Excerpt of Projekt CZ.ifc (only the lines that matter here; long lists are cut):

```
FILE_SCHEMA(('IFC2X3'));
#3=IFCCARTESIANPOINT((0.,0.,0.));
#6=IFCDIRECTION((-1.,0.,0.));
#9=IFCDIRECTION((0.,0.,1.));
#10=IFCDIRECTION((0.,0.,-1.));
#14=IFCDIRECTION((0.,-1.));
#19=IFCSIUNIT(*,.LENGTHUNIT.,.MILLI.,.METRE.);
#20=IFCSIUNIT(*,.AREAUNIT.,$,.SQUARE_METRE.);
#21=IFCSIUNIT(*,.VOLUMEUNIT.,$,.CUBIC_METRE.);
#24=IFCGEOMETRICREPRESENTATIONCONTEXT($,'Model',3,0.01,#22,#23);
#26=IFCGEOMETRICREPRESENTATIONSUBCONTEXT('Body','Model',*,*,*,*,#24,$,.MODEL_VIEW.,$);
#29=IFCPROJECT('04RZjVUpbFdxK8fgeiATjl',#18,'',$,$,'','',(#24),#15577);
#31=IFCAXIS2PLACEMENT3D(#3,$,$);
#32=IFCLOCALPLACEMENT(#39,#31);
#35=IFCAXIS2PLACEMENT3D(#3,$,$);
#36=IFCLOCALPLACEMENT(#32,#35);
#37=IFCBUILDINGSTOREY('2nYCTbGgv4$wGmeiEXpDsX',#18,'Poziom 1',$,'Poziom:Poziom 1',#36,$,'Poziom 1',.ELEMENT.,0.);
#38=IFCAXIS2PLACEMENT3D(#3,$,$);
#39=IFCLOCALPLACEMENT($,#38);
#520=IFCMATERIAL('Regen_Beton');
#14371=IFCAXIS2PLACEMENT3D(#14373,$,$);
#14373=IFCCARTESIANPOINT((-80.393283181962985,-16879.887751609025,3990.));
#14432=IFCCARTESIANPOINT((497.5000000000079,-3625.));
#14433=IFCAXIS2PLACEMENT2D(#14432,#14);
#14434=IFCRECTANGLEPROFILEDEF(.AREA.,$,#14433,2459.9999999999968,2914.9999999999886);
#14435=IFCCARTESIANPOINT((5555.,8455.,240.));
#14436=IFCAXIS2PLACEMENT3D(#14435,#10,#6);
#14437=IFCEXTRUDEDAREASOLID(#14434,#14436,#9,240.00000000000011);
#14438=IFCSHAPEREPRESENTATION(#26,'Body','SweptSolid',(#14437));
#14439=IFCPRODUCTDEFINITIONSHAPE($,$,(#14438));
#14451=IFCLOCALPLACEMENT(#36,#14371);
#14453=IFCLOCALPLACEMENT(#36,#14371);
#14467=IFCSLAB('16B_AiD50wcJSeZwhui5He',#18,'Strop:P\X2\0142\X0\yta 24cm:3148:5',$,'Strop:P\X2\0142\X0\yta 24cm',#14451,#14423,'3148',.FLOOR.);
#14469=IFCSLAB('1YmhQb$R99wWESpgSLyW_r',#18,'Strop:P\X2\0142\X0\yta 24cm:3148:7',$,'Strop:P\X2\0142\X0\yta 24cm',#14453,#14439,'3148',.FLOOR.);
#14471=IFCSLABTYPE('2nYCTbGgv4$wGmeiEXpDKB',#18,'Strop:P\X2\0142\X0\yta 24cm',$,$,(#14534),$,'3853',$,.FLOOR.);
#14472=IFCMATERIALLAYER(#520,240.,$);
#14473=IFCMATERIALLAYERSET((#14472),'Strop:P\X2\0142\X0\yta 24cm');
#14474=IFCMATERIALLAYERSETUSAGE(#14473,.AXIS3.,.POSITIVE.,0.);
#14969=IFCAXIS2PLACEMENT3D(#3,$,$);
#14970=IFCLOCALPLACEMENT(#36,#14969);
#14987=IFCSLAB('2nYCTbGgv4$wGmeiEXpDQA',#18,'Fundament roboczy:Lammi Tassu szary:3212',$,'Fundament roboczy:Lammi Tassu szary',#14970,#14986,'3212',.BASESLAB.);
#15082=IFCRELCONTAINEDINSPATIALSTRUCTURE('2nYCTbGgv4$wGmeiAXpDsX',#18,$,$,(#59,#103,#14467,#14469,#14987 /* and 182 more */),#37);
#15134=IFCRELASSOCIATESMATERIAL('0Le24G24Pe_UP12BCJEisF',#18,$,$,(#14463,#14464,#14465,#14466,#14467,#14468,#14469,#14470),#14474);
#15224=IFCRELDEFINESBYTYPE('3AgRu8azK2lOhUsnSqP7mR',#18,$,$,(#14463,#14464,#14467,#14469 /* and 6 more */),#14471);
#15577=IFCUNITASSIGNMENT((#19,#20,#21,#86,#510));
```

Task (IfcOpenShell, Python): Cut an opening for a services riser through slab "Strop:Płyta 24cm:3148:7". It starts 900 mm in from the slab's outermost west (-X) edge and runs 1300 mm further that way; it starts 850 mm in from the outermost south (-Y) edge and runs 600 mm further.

```python
import numpy as np
import ifcopenshell
import ifcopenshell.api.feature
import ifcopenshell.api.geometry
import ifcopenshell.api.root
import ifcopenshell.geom
import ifcopenshell.util.placement
import ifcopenshell.util.representation
import ifcopenshell.util.shape
import ifcopenshell.util.unit

model = ifcopenshell.open("Projekt CZ.ifc")
unit_scale = ifcopenshell.util.unit.calculate_unit_scale(model)
settings = ifcopenshell.geom.settings()


def volume(element):
    """Net volume in cubic metres, openings subtracted."""
    shape = ifcopenshell.geom.create_shape(settings, element)
    return ifcopenshell.util.shape.get_volume(shape.geometry)


slab = model.by_guid("1YmhQb$R99wWESpgSLyW_r")
before = volume(slab)

# Extent in the slab's own axes, in metres. The edges named are its -X and -Y sides.
slab_shape = ifcopenshell.geom.create_shape(settings, slab)
vertices = ifcopenshell.util.shape.get_vertices(slab_shape.geometry)
x_min, y_min, bottom = vertices.min(axis=0)
top = vertices[:, 2].max()

opening = ifcopenshell.api.root.create_entity(model, ifc_class="IfcOpeningElement", name="Services riser opening")
context = ifcopenshell.util.representation.get_context(model, "Model", "Body", "MODEL_VIEW")
width, depth = 1.3, 0.6
outline = [(0.0, 0.0), (width, 0.0), (width, depth), (0.0, depth), (0.0, 0.0)]
# Overshoot both faces by 50 mm so the cut is clean.
shape = ifcopenshell.api.geometry.add_slab_representation(
    model, context=context, depth=top - bottom + 0.1, polyline=outline
)
ifcopenshell.api.geometry.assign_representation(model, product=opening, representation=shape)

matrix = ifcopenshell.util.placement.get_local_placement(slab.ObjectPlacement)
matrix[:, 3] = matrix @ np.append(np.array([x_min + 0.9, y_min + 0.85, bottom - 0.05]) / unit_scale, 1.0)
ifcopenshell.api.geometry.edit_object_placement(model, product=opening, matrix=matrix, is_si=False)
ifcopenshell.api.feature.add_feature(model, feature=opening, element=slab)

after = volume(slab)

print(f"slab volume {before:.3f} -> {after:.3f} m3")

model.write("Projekt CZ_edited.ifc")
```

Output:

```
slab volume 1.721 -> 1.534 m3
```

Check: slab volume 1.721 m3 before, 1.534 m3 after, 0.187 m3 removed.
